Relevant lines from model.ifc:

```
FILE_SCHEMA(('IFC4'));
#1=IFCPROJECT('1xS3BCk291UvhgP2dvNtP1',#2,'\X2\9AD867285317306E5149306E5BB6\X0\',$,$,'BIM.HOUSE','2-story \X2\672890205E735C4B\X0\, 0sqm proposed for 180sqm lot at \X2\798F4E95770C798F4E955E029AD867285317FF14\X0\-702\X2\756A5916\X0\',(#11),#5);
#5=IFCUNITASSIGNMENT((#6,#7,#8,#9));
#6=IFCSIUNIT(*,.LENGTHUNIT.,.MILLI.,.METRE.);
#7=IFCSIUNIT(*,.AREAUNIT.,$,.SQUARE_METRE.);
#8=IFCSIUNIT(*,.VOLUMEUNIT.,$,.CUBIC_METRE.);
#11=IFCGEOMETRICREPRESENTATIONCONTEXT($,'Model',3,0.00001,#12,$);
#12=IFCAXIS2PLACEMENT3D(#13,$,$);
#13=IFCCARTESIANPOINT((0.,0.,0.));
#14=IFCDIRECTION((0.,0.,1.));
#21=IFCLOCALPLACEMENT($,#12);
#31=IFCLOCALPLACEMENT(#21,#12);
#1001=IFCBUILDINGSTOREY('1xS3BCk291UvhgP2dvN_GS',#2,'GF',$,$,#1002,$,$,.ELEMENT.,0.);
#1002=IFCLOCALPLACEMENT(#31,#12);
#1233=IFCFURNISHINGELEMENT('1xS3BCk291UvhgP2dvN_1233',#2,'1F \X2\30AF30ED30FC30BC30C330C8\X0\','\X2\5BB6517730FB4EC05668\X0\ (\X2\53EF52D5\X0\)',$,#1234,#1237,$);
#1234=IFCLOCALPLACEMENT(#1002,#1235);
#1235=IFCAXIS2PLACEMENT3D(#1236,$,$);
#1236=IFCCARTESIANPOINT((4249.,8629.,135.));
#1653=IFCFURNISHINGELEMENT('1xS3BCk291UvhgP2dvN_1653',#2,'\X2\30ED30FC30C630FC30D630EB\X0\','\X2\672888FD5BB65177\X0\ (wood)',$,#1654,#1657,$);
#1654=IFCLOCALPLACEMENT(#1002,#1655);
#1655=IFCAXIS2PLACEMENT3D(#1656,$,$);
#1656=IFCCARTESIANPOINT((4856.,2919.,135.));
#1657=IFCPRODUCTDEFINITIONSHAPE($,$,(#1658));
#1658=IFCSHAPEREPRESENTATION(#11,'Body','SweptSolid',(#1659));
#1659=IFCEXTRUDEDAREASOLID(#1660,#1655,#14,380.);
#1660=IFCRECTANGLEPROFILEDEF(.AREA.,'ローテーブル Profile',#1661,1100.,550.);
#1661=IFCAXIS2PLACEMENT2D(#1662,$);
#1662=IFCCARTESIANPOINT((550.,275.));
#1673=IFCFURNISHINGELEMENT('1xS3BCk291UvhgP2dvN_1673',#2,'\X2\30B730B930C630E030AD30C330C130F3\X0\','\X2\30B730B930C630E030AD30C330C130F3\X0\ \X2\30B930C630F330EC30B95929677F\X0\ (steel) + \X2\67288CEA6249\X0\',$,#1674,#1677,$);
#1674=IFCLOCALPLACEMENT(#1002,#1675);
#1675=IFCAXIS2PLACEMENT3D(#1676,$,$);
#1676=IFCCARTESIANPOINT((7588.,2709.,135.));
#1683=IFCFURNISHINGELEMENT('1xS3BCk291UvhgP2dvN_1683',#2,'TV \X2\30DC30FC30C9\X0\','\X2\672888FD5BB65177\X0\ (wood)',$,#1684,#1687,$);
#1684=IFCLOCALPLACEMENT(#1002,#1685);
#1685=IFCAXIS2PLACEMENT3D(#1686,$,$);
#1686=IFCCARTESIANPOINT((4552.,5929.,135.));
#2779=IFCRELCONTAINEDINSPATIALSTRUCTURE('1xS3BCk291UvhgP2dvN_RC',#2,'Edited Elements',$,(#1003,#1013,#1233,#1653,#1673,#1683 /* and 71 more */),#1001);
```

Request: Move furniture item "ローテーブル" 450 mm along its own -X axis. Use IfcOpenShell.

```python
import ifcopenshell
import ifcopenshell.api.geometry
import ifcopenshell.util.placement
import ifcopenshell.util.unit

model = ifcopenshell.open("model.ifc")
unit_scale = ifcopenshell.util.unit.calculate_unit_scale(model)

item = model.by_guid("1xS3BCk291UvhgP2dvN_1653")
matrix = ifcopenshell.util.placement.get_local_placement(item.ObjectPlacement)
matrix[:3, 3] -= matrix[:3, 0] * 0.45 / unit_scale
ifcopenshell.api.geometry.edit_object_placement(model, product=item, matrix=matrix, is_si=False)

print(ifcopenshell.util.placement.get_local_placement(item.ObjectPlacement).round(3) + 0.0)

model.write("model_rev.ifc")
```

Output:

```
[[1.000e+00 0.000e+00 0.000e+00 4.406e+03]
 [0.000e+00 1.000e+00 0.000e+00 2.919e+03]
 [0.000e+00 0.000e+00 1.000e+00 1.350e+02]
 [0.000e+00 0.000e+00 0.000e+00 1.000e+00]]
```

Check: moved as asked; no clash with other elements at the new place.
